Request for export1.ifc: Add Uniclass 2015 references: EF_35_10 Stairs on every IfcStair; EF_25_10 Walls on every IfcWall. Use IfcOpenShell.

First a look at what the model holds.

```python
import ifcopenshell

model = ifcopenshell.open("export1.ifc")
print(model.schema)
print("classifications:", [c.Name for c in model.by_type("IfcClassification")])
for ifc_class in ("IfcDoor", "IfcRoof", "IfcStair", "IfcWall", "IfcWindow"):
    print(ifc_class, len(model.by_type(ifc_class)))
```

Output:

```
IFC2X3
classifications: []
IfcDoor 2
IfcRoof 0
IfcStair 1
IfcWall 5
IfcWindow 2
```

```python
import ifcopenshell
import ifcopenshell.api.classification

model = ifcopenshell.open("export1.ifc")

# IFC2X3 requires Source and Edition and has no link from the project to the system.
system = model.create_entity("IfcClassification", Source="NBS", Edition="2015", Name="Uniclass 2015")

codes = {
    "IfcStair": ("EF_35_10", "Stairs"),
    "IfcWall": ("EF_25_10", "Walls"),
}
for ifc_class, (code, name) in codes.items():
    products = model.by_type(ifc_class)
    ifcopenshell.api.classification.add_reference(
        model, products=products, classification=system, identification=code, name=name
    )
    print(code, len(products))

model.write("export1_rev.ifc")
```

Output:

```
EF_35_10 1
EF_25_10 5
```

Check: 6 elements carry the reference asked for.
